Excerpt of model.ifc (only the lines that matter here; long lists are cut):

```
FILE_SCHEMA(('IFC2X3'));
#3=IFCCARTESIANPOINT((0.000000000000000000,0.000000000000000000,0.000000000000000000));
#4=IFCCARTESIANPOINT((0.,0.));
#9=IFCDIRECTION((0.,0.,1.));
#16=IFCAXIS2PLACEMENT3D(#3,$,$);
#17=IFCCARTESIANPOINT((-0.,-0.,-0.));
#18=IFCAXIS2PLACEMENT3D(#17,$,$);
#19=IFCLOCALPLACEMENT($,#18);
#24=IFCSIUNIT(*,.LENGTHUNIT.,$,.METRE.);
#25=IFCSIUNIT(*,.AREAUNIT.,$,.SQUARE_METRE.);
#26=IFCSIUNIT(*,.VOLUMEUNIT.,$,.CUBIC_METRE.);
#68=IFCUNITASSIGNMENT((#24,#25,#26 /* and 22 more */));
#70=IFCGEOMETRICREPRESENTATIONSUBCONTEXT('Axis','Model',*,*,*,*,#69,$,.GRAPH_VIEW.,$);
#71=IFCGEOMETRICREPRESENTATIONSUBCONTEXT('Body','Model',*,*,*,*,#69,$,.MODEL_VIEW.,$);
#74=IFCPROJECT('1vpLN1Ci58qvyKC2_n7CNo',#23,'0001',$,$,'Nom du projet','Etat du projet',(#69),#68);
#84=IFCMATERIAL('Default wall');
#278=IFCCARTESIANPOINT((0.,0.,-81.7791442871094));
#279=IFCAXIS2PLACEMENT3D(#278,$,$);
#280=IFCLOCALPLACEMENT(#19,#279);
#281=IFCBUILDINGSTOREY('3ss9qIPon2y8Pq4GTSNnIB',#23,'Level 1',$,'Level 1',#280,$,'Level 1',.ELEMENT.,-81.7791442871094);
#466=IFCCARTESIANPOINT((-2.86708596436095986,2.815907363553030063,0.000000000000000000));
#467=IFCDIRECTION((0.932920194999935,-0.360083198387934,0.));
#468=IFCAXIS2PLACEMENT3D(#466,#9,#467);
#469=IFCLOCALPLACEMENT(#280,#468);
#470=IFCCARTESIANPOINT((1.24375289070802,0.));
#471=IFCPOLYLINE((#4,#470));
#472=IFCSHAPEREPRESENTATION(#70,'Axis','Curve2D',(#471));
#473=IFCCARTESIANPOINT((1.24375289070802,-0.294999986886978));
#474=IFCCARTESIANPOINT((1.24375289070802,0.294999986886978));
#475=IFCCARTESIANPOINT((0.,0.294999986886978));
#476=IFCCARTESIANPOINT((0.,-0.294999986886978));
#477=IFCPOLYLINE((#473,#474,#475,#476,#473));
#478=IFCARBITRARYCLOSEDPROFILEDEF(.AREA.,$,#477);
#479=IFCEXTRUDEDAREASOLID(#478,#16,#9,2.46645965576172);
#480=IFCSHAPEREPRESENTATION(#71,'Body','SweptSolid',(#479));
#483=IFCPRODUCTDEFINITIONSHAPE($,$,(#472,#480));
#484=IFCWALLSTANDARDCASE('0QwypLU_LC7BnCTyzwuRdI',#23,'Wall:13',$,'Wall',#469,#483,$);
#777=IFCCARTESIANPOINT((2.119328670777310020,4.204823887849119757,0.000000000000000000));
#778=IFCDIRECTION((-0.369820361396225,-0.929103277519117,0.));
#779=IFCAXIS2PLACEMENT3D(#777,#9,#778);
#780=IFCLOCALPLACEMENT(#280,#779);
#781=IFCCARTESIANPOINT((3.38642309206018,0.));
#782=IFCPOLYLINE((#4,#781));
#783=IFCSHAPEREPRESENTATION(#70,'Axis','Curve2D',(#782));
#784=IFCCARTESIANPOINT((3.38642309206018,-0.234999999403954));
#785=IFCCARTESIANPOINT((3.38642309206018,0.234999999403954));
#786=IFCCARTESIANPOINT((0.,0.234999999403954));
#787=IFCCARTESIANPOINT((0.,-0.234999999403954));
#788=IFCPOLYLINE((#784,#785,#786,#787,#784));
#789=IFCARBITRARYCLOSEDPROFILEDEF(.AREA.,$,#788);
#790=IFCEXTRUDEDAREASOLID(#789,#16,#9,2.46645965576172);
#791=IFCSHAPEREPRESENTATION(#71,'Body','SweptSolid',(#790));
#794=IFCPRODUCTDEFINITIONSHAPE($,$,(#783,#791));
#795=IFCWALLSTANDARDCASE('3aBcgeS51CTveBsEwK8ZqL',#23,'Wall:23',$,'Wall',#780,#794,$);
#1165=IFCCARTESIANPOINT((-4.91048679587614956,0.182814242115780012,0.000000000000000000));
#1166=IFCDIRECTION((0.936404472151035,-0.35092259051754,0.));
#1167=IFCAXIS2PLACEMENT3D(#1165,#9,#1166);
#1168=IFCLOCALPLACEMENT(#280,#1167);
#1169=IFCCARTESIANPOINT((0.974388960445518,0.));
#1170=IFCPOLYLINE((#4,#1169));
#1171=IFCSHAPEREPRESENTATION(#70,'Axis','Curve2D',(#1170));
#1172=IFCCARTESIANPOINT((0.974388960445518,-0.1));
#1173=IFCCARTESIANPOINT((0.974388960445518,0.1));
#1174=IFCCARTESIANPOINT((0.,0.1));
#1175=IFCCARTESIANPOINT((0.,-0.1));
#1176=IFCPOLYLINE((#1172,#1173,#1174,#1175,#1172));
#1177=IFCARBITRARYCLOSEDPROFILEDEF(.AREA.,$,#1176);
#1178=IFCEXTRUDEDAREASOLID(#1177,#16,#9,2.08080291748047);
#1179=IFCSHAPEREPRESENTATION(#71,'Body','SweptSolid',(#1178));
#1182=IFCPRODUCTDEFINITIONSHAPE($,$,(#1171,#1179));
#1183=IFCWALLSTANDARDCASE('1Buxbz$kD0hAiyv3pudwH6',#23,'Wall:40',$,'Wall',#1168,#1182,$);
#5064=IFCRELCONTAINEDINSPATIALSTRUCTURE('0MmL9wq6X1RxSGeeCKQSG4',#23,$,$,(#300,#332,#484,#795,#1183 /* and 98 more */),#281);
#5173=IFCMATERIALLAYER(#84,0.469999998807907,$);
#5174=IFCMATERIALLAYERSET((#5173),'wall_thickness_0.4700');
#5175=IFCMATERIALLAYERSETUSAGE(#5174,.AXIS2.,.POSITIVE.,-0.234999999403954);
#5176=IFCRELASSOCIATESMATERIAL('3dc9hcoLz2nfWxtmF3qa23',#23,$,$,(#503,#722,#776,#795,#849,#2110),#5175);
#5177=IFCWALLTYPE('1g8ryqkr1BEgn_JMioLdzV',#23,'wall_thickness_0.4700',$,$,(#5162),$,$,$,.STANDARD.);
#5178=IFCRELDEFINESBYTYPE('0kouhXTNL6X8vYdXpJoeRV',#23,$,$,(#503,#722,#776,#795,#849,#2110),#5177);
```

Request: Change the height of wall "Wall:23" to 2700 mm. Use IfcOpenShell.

```python
import ifcopenshell
import ifcopenshell.geom
import ifcopenshell.util.representation
import ifcopenshell.util.shape

model = ifcopenshell.open("model.ifc")
settings = ifcopenshell.geom.settings()


def volume(element):
    """Net volume in cubic metres, openings subtracted."""
    shape = ifcopenshell.geom.create_shape(settings, element)
    return ifcopenshell.util.shape.get_volume(shape.geometry)


wall = model.by_guid("3aBcgeS51CTveBsEwK8ZqL")
before = volume(wall)

body = ifcopenshell.util.representation.get_representation(wall, "Model", "Body")
solid = body.Items[0]
old_height = solid.Depth
solid.Depth = 2.7
after = volume(wall)

print(f"height {old_height:g} -> {solid.Depth:g}, volume {before:.3f} -> {after:.3f} m3")

model.write("model_v2.ifc")
```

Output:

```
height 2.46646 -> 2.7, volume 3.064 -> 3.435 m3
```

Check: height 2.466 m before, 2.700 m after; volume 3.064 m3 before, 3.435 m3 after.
